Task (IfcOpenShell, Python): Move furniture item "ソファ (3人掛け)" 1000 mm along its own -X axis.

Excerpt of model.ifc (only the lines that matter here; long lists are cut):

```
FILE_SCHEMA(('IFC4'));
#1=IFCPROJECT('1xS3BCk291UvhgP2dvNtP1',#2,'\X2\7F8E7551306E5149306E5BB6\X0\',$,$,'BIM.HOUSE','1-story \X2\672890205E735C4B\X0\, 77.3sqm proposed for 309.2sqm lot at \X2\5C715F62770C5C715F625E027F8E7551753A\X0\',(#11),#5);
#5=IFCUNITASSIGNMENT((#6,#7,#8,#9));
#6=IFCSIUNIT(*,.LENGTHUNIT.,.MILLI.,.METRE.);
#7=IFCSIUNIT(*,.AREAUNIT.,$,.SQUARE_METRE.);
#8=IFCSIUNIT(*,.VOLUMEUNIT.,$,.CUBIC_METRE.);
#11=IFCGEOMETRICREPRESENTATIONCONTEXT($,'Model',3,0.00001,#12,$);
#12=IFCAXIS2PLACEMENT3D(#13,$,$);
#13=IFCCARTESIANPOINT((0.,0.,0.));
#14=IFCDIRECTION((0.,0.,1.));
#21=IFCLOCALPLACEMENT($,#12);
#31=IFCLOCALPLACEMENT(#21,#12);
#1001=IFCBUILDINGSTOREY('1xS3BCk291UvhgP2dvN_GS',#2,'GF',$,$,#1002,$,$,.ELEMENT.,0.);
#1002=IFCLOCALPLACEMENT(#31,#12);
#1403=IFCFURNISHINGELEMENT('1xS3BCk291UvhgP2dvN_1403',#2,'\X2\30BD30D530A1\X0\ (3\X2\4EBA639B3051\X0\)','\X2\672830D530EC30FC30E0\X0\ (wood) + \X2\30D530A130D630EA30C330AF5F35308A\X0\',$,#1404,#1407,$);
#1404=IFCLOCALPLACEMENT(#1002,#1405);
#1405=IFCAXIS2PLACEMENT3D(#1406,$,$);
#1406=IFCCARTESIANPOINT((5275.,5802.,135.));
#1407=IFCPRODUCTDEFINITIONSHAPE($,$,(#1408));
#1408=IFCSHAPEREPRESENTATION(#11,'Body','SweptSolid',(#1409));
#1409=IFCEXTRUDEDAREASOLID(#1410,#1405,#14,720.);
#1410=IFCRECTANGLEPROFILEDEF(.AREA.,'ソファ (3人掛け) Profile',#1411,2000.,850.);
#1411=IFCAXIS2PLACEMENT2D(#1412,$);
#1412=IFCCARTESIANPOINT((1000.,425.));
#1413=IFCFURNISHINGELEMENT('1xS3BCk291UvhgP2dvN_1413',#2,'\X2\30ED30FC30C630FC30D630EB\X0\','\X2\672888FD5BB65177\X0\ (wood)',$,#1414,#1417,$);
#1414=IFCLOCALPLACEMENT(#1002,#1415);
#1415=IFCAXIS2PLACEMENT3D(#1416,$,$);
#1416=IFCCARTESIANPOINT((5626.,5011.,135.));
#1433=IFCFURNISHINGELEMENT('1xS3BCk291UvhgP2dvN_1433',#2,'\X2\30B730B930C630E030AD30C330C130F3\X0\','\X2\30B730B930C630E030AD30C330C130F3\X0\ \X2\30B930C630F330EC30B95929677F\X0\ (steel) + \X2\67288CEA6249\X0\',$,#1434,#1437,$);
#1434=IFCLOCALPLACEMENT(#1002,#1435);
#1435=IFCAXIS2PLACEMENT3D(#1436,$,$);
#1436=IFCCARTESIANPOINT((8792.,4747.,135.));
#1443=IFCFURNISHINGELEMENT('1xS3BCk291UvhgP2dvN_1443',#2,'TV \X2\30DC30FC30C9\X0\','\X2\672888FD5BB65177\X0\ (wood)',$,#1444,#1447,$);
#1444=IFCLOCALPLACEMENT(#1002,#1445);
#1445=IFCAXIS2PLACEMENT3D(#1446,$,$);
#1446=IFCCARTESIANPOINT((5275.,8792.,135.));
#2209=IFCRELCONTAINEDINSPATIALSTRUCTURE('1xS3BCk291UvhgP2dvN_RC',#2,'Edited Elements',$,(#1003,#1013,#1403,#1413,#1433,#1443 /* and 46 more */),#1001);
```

```python
import ifcopenshell
import ifcopenshell.api.geometry
import ifcopenshell.util.placement
import ifcopenshell.util.unit

model = ifcopenshell.open("model.ifc")
unit_scale = ifcopenshell.util.unit.calculate_unit_scale(model)

item = model.by_guid("1xS3BCk291UvhgP2dvN_1403")
matrix = ifcopenshell.util.placement.get_local_placement(item.ObjectPlacement)
matrix[:3, 3] -= matrix[:3, 0] * 1 / unit_scale
ifcopenshell.api.geometry.edit_object_placement(model, product=item, matrix=matrix, is_si=False)

print(ifcopenshell.util.placement.get_local_placement(item.ObjectPlacement).round(3) + 0.0)

model.write("model_updated.ifc")
```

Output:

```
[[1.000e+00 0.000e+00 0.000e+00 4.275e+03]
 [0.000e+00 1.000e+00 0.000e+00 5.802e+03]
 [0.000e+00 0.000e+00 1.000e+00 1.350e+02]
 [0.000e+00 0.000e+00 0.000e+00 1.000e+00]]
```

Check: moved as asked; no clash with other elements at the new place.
